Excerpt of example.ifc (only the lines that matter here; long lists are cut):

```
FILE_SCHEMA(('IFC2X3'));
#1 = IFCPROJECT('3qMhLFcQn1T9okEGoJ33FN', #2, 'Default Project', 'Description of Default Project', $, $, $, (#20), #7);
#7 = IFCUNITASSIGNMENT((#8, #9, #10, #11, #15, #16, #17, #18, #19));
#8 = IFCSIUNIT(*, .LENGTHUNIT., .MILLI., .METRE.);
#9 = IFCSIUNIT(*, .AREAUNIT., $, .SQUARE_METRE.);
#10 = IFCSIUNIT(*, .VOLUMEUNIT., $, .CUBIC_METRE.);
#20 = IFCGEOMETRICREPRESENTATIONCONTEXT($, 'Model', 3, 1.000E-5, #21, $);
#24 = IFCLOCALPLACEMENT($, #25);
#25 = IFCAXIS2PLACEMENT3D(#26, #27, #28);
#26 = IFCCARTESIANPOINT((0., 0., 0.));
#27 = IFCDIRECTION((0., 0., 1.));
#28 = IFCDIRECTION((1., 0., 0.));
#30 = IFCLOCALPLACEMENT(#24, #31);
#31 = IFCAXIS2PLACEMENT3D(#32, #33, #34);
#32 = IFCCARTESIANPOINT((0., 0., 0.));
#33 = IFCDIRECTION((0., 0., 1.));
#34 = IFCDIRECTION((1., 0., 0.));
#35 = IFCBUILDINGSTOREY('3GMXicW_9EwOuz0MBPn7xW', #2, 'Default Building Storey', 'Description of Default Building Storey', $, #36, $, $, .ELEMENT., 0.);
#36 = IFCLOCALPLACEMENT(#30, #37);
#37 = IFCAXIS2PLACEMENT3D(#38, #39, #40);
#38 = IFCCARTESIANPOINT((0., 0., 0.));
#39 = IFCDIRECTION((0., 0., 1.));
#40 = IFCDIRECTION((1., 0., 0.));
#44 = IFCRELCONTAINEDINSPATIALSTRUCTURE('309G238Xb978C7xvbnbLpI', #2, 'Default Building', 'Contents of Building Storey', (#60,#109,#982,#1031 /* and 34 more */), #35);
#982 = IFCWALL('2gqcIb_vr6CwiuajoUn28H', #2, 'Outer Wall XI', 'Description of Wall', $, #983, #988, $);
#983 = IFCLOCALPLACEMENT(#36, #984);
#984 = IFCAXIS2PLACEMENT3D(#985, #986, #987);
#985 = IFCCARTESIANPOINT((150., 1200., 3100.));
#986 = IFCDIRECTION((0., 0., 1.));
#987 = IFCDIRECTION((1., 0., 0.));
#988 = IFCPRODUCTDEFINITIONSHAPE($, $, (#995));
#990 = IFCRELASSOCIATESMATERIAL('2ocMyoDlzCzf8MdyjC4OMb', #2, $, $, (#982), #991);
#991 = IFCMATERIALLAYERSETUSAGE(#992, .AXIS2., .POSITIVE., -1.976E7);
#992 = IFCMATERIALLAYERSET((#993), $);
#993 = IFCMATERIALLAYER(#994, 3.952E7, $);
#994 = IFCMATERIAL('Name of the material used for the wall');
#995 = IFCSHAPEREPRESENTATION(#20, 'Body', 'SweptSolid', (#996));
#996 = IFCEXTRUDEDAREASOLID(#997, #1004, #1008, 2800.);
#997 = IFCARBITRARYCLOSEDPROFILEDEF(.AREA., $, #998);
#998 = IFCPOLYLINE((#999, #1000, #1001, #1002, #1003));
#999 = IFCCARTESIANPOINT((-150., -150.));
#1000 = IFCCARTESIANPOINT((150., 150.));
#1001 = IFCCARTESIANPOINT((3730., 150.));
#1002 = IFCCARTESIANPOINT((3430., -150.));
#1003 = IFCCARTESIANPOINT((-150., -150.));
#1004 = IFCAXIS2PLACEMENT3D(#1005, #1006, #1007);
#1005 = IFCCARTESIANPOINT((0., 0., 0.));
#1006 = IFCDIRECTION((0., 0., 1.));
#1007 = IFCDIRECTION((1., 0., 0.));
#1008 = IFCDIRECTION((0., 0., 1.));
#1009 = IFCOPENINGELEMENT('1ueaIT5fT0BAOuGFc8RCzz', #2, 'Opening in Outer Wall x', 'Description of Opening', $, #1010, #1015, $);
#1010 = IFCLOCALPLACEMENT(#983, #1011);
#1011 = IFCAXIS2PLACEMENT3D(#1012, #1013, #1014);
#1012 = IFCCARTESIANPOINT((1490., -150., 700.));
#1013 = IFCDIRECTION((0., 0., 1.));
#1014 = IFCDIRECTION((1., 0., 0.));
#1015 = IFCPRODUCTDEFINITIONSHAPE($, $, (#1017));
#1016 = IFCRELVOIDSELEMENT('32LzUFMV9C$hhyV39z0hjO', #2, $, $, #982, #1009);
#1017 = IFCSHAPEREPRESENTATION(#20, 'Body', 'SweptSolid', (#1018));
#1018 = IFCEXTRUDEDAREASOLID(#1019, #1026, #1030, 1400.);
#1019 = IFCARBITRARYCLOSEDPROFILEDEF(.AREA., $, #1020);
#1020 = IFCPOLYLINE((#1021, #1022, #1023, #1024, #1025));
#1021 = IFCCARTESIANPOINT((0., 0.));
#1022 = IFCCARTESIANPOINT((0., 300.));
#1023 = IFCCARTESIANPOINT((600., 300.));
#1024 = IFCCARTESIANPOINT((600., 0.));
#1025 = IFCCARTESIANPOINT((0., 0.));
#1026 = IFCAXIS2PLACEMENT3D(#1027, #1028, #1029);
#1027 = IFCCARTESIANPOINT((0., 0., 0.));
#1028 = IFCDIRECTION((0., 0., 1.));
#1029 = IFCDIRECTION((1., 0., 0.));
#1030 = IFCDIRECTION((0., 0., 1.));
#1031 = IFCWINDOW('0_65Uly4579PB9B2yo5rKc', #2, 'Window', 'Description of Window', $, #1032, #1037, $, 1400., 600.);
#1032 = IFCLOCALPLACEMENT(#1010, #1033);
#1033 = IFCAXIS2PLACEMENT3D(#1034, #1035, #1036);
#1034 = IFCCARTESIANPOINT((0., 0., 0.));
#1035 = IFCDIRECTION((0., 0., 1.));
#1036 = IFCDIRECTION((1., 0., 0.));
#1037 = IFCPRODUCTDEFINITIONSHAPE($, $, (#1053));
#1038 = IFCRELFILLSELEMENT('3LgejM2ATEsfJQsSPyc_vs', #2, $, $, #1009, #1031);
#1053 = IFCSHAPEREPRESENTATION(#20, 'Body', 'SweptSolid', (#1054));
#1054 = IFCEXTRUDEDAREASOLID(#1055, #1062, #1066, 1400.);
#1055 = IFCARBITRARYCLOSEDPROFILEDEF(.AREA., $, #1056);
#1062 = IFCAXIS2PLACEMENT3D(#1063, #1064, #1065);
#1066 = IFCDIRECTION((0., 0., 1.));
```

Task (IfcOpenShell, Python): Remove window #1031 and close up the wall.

```python
import ifcopenshell
import ifcopenshell.api.feature
import ifcopenshell.api.root
import ifcopenshell.geom
import ifcopenshell.util.shape

model = ifcopenshell.open("example.ifc")
settings = ifcopenshell.geom.settings()


def volume(element):
    """Net volume in cubic metres, openings subtracted."""
    shape = ifcopenshell.geom.create_shape(settings, element)
    return ifcopenshell.util.shape.get_volume(shape.geometry)


window = model.by_guid("0_65Uly4579PB9B2yo5rKc")
opening = window.FillsVoids[0].RelatingOpeningElement
wall = opening.VoidsElements[0].RelatingBuildingElement
before = volume(wall)

ifcopenshell.api.root.remove_product(model, product=window)
ifcopenshell.api.feature.remove_feature(model, feature=opening)

after = volume(wall)

print(f"wall volume {before:.3f} -> {after:.3f} m3")

model.write("example_edited.ifc")
```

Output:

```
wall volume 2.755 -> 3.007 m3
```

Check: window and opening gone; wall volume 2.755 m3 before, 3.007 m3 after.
